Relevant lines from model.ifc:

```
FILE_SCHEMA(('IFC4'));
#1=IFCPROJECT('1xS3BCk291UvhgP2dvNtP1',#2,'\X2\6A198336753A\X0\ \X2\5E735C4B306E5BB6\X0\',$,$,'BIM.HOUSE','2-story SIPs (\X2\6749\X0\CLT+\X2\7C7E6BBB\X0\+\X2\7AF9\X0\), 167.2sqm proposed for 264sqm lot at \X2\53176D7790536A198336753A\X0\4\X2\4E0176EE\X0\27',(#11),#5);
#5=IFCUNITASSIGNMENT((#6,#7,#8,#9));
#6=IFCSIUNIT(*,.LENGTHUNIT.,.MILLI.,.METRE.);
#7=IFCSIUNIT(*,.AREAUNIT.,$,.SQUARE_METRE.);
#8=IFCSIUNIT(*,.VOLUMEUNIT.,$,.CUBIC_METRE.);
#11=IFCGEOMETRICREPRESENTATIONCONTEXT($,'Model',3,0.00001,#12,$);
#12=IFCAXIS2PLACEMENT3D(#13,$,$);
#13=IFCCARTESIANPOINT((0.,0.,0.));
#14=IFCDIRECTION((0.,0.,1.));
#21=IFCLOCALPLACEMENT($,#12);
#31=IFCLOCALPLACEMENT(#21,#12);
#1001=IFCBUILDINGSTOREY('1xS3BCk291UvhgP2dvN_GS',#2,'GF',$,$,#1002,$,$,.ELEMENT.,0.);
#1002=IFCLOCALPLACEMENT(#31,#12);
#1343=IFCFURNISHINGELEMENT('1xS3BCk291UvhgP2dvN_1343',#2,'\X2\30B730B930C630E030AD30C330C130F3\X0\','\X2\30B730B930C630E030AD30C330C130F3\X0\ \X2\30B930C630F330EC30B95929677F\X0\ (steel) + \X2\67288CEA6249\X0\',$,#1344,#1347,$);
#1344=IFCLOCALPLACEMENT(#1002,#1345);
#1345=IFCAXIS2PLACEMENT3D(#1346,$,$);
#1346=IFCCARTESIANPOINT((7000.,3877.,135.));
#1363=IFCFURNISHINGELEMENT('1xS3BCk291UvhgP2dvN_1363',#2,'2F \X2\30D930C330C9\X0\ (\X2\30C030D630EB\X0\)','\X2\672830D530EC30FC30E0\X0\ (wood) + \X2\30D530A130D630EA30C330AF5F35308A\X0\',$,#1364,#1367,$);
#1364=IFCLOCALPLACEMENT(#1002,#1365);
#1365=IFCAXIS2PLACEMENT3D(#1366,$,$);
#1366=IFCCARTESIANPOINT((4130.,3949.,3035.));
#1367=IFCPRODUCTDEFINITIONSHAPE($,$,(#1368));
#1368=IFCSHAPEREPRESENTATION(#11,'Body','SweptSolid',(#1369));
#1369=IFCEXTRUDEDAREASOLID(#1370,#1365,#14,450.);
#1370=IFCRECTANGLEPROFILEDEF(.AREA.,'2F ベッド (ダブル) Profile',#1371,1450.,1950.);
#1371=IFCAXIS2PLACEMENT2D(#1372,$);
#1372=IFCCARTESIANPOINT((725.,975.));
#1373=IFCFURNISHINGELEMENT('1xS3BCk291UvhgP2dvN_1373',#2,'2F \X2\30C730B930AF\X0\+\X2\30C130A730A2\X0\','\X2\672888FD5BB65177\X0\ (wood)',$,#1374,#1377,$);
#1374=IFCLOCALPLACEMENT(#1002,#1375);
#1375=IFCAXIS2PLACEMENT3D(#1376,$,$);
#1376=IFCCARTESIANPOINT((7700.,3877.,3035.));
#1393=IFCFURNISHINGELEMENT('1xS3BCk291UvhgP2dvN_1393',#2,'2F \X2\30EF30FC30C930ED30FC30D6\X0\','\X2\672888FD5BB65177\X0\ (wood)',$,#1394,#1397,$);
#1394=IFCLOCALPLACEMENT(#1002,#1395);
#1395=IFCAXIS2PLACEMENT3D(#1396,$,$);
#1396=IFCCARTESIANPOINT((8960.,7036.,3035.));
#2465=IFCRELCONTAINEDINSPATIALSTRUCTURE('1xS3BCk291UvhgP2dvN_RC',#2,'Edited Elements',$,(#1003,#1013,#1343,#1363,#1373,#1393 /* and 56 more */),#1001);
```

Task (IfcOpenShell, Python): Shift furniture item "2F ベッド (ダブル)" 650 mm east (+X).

```python
import ifcopenshell
import ifcopenshell.api.geometry
import ifcopenshell.util.placement
import ifcopenshell.util.unit

model = ifcopenshell.open("model.ifc")
unit_scale = ifcopenshell.util.unit.calculate_unit_scale(model)

item = model.by_id(1363)
matrix = ifcopenshell.util.placement.get_local_placement(item.ObjectPlacement)
matrix[0, 3] += 0.65 / unit_scale
ifcopenshell.api.geometry.edit_object_placement(model, product=item, matrix=matrix, is_si=False)

print(ifcopenshell.util.placement.get_local_placement(item.ObjectPlacement).round(3) + 0.0)

model.write("model_edited.ifc")
```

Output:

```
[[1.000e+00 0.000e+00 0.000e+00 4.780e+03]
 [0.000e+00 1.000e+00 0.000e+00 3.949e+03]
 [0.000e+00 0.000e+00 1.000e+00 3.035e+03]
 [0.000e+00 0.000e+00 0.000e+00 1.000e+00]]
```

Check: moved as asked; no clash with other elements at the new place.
